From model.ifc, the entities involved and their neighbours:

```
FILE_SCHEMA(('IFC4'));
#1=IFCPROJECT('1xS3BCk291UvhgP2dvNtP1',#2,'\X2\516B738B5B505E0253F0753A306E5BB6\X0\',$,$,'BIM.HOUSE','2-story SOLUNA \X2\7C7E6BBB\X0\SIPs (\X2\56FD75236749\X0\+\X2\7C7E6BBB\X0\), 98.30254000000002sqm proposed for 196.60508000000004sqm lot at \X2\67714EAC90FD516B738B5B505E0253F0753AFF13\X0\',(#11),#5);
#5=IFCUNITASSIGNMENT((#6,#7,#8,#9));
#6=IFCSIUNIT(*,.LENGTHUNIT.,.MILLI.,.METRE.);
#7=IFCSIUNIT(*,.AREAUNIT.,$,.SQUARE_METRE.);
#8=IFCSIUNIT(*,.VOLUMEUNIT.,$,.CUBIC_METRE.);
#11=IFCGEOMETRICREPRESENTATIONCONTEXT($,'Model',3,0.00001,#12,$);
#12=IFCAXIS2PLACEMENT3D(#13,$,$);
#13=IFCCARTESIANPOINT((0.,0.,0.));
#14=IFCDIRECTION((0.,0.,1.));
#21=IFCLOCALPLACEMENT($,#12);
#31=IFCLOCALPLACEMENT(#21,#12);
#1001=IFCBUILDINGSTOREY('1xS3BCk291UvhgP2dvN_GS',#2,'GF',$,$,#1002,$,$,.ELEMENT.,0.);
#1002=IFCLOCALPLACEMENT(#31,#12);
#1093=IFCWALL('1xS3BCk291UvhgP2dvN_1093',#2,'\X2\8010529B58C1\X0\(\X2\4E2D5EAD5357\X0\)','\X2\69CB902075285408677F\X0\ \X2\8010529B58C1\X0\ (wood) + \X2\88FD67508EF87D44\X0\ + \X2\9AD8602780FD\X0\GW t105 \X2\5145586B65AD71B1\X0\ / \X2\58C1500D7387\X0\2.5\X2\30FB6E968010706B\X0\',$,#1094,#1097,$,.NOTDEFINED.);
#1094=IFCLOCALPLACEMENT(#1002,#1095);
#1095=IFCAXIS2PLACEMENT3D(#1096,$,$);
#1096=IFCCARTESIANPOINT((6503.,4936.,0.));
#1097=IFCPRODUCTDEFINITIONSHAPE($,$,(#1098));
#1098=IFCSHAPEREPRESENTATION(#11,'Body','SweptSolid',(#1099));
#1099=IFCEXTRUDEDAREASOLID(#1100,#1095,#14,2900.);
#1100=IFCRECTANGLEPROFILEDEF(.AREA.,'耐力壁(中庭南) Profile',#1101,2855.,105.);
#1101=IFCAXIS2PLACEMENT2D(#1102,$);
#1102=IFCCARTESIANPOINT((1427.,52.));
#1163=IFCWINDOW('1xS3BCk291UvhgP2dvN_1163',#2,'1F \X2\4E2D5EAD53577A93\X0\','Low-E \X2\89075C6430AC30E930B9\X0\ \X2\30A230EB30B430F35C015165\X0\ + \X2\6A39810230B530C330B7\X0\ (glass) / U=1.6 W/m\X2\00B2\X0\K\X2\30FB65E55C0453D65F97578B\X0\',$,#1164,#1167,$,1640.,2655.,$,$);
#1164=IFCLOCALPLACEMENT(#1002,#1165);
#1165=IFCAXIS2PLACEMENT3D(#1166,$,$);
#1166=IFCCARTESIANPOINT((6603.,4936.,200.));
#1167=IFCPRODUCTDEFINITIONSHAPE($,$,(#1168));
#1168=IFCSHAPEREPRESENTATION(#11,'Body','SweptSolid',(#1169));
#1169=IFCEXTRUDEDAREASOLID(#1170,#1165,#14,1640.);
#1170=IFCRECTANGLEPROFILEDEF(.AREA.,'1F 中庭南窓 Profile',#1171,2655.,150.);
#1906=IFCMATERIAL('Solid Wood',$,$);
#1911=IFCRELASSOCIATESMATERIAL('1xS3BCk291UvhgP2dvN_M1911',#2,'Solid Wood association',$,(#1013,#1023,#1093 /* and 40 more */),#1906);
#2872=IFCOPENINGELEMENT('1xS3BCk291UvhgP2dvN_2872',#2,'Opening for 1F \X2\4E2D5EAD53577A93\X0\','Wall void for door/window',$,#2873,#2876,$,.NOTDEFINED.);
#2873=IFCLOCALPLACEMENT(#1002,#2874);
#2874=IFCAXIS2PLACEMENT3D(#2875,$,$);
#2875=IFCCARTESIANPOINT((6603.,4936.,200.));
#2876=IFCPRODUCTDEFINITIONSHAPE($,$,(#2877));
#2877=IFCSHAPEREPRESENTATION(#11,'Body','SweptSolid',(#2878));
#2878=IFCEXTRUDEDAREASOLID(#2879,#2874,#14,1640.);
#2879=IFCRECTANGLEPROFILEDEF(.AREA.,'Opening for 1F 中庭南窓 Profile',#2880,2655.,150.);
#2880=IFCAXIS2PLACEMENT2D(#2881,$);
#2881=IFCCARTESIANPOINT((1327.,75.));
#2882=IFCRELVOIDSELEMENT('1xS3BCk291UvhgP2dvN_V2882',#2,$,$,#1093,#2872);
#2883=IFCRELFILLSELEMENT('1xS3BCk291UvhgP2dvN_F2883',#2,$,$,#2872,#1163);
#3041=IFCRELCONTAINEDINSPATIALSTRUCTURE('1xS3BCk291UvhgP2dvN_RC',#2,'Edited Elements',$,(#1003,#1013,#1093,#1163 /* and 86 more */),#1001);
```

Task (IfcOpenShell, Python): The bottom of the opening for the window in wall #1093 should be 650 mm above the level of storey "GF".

```python
import numpy as np
import ifcopenshell
import ifcopenshell.api.geometry
import ifcopenshell.geom
import ifcopenshell.util.element
import ifcopenshell.util.placement
import ifcopenshell.util.shape
import ifcopenshell.util.unit

model = ifcopenshell.open("model.ifc")
unit_scale = ifcopenshell.util.unit.calculate_unit_scale(model)

window = model.by_guid("1xS3BCk291UvhgP2dvN_1163")
opening = window.FillsVoids[0].RelatingOpeningElement
storey = ifcopenshell.util.element.get_container(window, ifc_class="IfcBuildingStorey")
level = ifcopenshell.util.placement.get_local_placement(storey.ObjectPlacement)[2, 3]

# The opening's origin need not be at the sill, so measure its lowest point.
shape = ifcopenshell.geom.create_shape(ifcopenshell.geom.settings(), opening)
bottom = ifcopenshell.util.shape.get_shape_bottom_elevation(shape, shape.geometry) / unit_scale
dz = level + 0.65 / unit_scale - bottom

shift = np.array([0.0, 0.0, dz])
# The window is not placed relative to its opening, so move both.
for product in (opening, window):
    matrix = ifcopenshell.util.placement.get_local_placement(product.ObjectPlacement)
    matrix[:3, 3] += shift
    ifcopenshell.api.geometry.edit_object_placement(model, product=product, matrix=matrix, is_si=False)

print(f"moved by {dz * unit_scale:+.3f} m")

model.write("model_updated.ifc")
```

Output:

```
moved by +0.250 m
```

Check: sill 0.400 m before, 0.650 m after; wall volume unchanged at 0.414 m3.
